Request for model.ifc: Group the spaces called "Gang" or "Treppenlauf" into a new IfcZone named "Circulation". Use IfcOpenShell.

First a look at what the model holds.

```python
import ifcopenshell

model = ifcopenshell.open("model.ifc")
print(model.schema)
seen = {}
for space in model.by_type("IfcSpace"):
    seen[space.LongName] = seen.get(space.LongName, 0) + 1
for name, count in sorted(seen.items(), key=str):
    print(count, "x", name)
print("zones:", [z.Name for z in model.by_type("IfcZone")][:20])
```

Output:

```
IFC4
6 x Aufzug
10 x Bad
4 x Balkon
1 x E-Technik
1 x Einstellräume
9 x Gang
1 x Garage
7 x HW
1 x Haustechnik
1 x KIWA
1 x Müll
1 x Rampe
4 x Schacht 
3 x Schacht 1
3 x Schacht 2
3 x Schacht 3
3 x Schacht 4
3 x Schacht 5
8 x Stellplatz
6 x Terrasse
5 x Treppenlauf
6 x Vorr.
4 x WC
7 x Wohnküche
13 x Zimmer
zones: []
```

```python
import ifcopenshell
import ifcopenshell.api.group
import ifcopenshell.api.root

model = ifcopenshell.open("model.ifc")

names = {"Gang", "Treppenlauf"}
spaces = [s for s in model.by_type("IfcSpace") if s.LongName in names]

zone = ifcopenshell.api.root.create_entity(model, ifc_class="IfcZone", name="Circulation")
ifcopenshell.api.group.assign_group(model, products=spaces, group=zone)
print(len(spaces), "spaces in", zone.Name)

model.write("model-out.ifc")
```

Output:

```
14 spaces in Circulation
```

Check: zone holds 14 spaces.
